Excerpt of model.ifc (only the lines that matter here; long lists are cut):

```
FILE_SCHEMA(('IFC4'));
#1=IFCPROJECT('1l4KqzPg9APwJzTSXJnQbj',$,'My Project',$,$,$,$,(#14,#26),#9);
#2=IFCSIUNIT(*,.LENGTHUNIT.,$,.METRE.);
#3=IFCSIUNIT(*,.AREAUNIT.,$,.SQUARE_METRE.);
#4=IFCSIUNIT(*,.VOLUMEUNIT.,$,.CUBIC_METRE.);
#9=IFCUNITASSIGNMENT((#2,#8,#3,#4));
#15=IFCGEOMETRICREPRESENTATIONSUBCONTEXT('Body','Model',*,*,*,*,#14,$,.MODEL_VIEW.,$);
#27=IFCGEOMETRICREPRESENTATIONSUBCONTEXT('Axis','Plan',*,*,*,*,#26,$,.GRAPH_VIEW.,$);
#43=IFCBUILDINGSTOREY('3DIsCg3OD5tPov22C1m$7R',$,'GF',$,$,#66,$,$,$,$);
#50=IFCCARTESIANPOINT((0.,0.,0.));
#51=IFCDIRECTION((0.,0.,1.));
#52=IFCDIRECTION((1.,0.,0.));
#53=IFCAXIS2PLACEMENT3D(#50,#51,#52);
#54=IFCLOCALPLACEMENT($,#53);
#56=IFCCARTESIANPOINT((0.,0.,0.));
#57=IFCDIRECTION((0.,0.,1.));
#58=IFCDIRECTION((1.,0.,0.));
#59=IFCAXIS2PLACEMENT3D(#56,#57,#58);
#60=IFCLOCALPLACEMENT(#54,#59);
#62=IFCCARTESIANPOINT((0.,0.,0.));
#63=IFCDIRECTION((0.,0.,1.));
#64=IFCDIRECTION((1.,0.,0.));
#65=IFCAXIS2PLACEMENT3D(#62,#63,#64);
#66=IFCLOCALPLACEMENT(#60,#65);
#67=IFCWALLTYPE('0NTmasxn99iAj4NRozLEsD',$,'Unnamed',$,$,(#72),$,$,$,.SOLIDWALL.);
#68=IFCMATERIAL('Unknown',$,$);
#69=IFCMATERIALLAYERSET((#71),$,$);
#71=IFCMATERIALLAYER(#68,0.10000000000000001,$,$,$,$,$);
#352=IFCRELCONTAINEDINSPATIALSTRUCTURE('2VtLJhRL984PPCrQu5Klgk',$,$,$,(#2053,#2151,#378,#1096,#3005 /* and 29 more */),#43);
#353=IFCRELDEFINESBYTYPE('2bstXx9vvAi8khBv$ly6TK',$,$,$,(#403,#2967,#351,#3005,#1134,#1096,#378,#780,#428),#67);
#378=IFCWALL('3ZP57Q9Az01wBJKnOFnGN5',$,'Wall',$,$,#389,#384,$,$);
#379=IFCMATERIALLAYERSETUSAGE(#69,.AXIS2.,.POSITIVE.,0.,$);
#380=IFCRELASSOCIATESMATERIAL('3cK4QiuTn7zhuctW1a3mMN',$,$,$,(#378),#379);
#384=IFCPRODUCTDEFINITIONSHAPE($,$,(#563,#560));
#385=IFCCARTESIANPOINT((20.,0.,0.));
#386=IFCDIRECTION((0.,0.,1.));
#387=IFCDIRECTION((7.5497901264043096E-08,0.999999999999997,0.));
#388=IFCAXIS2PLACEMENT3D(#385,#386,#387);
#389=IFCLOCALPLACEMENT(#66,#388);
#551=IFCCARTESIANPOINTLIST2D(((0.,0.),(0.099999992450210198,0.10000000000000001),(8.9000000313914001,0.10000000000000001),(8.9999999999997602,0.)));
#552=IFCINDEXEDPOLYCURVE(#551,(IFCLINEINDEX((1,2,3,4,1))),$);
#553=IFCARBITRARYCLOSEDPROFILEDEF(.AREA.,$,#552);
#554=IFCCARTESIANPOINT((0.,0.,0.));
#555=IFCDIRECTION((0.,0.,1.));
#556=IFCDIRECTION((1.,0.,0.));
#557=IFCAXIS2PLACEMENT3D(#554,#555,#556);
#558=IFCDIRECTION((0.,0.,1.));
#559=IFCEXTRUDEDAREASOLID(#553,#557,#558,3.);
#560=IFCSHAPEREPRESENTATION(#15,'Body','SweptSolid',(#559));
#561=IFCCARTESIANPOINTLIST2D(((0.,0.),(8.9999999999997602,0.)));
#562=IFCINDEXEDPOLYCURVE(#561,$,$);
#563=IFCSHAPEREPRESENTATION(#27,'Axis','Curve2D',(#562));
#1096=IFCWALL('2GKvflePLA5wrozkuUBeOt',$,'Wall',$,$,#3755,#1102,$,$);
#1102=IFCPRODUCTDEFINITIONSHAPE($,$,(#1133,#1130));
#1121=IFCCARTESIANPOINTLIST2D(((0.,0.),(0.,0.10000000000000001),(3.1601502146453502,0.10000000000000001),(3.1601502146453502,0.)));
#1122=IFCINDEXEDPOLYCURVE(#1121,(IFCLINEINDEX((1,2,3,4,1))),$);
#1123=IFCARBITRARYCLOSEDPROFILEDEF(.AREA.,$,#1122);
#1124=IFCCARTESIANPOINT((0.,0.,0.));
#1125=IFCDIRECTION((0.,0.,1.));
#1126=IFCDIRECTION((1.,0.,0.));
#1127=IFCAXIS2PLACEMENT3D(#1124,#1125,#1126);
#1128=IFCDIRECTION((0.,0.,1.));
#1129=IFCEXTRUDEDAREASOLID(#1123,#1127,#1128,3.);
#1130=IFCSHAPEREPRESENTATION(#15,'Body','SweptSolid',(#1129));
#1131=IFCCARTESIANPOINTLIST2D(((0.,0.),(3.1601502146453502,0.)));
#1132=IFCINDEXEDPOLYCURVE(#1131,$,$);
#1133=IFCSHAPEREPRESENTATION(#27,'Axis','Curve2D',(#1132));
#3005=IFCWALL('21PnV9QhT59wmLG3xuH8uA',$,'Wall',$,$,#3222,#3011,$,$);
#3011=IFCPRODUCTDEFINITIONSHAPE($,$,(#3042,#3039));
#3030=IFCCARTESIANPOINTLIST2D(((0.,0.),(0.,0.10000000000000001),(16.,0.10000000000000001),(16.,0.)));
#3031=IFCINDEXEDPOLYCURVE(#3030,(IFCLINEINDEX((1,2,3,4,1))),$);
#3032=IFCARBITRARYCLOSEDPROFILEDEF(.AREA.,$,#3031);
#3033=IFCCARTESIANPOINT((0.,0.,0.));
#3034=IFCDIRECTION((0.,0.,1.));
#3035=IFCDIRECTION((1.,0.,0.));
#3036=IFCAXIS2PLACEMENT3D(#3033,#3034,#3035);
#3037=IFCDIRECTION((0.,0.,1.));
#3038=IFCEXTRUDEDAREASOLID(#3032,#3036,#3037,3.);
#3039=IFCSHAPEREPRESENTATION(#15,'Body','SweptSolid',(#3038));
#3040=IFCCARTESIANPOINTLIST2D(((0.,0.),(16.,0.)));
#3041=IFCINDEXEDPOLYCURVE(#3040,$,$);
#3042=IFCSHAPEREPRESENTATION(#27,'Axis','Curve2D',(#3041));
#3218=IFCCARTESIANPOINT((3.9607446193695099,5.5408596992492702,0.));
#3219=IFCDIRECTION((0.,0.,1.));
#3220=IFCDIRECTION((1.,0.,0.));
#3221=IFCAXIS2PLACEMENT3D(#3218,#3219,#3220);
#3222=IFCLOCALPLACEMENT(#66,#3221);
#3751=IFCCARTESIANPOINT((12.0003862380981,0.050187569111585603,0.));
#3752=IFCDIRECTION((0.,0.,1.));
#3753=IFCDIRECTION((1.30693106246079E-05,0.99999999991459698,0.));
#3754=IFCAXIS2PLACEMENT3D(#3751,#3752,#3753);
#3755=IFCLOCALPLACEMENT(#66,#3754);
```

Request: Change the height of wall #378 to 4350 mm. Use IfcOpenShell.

```python
import ifcopenshell
import ifcopenshell.geom
import ifcopenshell.util.representation
import ifcopenshell.util.shape

model = ifcopenshell.open("model.ifc")
settings = ifcopenshell.geom.settings()


def volume(element):
    """Net volume in cubic metres, openings subtracted."""
    shape = ifcopenshell.geom.create_shape(settings, element)
    return ifcopenshell.util.shape.get_volume(shape.geometry)


wall = model.by_guid("3ZP57Q9Az01wBJKnOFnGN5")
before = volume(wall)

body = ifcopenshell.util.representation.get_representation(wall, "Model", "Body")
solid = body.Items[0]
old_height = solid.Depth
solid.Depth = 4.35
after = volume(wall)

print(f"height {old_height:g} -> {solid.Depth:g}, volume {before:.3f} -> {after:.3f} m3")

model.write("model-out.ifc")
```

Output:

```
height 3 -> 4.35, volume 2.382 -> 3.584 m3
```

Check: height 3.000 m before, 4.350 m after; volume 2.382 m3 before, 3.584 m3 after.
